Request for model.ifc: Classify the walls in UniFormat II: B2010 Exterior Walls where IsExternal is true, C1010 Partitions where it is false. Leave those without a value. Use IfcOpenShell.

First a look at what the model holds.

```python
import ifcopenshell
import ifcopenshell.util.element

model = ifcopenshell.open("model.ifc")
print(model.schema)
print("classifications:", [c.Name for c in model.by_type("IfcClassification")])
values = [ifcopenshell.util.element.get_pset(e, "Pset_WallCommon", "IsExternal") for e in model.by_type("IfcWall")]
for value in (True, False, None):
    print("IsExternal", value, values.count(value))
```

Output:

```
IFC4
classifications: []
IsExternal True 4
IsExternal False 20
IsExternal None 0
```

```python
import ifcopenshell
import ifcopenshell.api.classification
import ifcopenshell.util.element

model = ifcopenshell.open("model.ifc")

system = ifcopenshell.api.classification.add_classification(model, classification="UniFormat II")

walls = model.by_type("IfcWall")
external = {e: ifcopenshell.util.element.get_pset(e, "Pset_WallCommon", "IsExternal") for e in walls}
for flag, code, name in ((True, "B2010", "Exterior Walls"), (False, "C1010", "Partitions")):
    products = [e for e in walls if external[e] is flag]
    ifcopenshell.api.classification.add_reference(
        model, products=products, classification=system, identification=code, name=name
    )
    print(code, len(products))

model.write("model_v2.ifc")
```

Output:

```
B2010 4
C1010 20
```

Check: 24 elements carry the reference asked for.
